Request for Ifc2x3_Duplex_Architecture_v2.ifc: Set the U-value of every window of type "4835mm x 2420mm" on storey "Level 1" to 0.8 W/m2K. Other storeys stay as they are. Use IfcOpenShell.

First a look at what the model holds.

```python
import ifcopenshell
import ifcopenshell.util.element

model = ifcopenshell.open("Ifc2x3_Duplex_Architecture_v2.ifc")
print(model.schema)
storey = next(s for s in model.by_type("IfcBuildingStorey") if s.Name == "Level 1")
windows = [e for e in ifcopenshell.util.element.get_decomposition(storey) if e.is_a("IfcWindow")]
seen = {}
for e in windows:
    element_type = ifcopenshell.util.element.get_type(e)
    key = (element_type.Name if element_type != e and element_type else None, ifcopenshell.util.element.get_pset(e, "Pset_WindowCommon", "ThermalTransmittance"))
    seen[key] = seen.get(key, 0) + 1
for (name, value), count in sorted(seen.items(), key=str):
    print(count, "x", name, "|", value)
```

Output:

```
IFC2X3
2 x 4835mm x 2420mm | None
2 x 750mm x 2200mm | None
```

```python
import ifcopenshell
import ifcopenshell.api.pset
import ifcopenshell.util.element

model = ifcopenshell.open("Ifc2x3_Duplex_Architecture_v2.ifc")

storey = next(s for s in model.by_type("IfcBuildingStorey") if s.Name == "Level 1")
windows = [e for e in ifcopenshell.util.element.get_decomposition(storey) if e.is_a("IfcWindow")]

count = 0
for e in windows:
    element_type = ifcopenshell.util.element.get_type(e)
    if element_type in (None, e) or element_type.Name != "4835mm x 2420mm":
        continue
    # add_pset returns the element's existing set when there is one.
    pset = ifcopenshell.api.pset.add_pset(model, product=e, name="Pset_WindowCommon")
    ifcopenshell.api.pset.edit_pset(model, pset=pset, properties={"ThermalTransmittance": 0.8})
    count += 1

print(count, "windows updated")

model.write("Ifc2x3_Duplex_Architecture_v2_rev.ifc")
```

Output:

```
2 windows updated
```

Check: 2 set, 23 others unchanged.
